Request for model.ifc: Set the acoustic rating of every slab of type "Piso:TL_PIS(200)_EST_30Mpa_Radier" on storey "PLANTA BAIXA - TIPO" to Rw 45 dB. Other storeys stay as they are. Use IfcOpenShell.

First a look at what the model holds.

```python
import ifcopenshell
import ifcopenshell.util.element

model = ifcopenshell.open("model.ifc")
print(model.schema)
storey = next(s for s in model.by_type("IfcBuildingStorey") if s.Name == "PLANTA BAIXA - TIPO")
slabs = [e for e in ifcopenshell.util.element.get_decomposition(storey) if e.is_a("IfcSlab")]
seen = {}
for e in slabs:
    element_type = ifcopenshell.util.element.get_type(e)
    key = (element_type.Name if element_type != e and element_type else None, ifcopenshell.util.element.get_pset(e, "Pset_SlabCommon", "AcousticRating"))
    seen[key] = seen.get(key, 0) + 1
for (name, value), count in sorted(seen.items(), key=str):
    print(count, "x", name, "|", value)
```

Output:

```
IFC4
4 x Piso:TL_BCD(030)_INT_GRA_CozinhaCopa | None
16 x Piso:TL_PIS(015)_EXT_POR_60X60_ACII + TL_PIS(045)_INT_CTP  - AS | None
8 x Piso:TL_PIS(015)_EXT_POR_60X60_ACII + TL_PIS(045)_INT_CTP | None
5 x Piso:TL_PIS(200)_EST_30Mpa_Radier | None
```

```python
import ifcopenshell
import ifcopenshell.api.pset
import ifcopenshell.util.element

model = ifcopenshell.open("model.ifc")

storey = next(s for s in model.by_type("IfcBuildingStorey") if s.Name == "PLANTA BAIXA - TIPO")
slabs = [e for e in ifcopenshell.util.element.get_decomposition(storey) if e.is_a("IfcSlab")]

count = 0
for e in slabs:
    element_type = ifcopenshell.util.element.get_type(e)
    if element_type in (None, e) or element_type.Name != "Piso:TL_PIS(200)_EST_30Mpa_Radier":
        continue
    # add_pset returns the element's existing set when there is one.
    pset = ifcopenshell.api.pset.add_pset(model, product=e, name="Pset_SlabCommon")
    ifcopenshell.api.pset.edit_pset(model, pset=pset, properties={"AcousticRating": "Rw 45 dB"})
    count += 1

print(count, "slabs updated")

model.write("model-out.ifc")
```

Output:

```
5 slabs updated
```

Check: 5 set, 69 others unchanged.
